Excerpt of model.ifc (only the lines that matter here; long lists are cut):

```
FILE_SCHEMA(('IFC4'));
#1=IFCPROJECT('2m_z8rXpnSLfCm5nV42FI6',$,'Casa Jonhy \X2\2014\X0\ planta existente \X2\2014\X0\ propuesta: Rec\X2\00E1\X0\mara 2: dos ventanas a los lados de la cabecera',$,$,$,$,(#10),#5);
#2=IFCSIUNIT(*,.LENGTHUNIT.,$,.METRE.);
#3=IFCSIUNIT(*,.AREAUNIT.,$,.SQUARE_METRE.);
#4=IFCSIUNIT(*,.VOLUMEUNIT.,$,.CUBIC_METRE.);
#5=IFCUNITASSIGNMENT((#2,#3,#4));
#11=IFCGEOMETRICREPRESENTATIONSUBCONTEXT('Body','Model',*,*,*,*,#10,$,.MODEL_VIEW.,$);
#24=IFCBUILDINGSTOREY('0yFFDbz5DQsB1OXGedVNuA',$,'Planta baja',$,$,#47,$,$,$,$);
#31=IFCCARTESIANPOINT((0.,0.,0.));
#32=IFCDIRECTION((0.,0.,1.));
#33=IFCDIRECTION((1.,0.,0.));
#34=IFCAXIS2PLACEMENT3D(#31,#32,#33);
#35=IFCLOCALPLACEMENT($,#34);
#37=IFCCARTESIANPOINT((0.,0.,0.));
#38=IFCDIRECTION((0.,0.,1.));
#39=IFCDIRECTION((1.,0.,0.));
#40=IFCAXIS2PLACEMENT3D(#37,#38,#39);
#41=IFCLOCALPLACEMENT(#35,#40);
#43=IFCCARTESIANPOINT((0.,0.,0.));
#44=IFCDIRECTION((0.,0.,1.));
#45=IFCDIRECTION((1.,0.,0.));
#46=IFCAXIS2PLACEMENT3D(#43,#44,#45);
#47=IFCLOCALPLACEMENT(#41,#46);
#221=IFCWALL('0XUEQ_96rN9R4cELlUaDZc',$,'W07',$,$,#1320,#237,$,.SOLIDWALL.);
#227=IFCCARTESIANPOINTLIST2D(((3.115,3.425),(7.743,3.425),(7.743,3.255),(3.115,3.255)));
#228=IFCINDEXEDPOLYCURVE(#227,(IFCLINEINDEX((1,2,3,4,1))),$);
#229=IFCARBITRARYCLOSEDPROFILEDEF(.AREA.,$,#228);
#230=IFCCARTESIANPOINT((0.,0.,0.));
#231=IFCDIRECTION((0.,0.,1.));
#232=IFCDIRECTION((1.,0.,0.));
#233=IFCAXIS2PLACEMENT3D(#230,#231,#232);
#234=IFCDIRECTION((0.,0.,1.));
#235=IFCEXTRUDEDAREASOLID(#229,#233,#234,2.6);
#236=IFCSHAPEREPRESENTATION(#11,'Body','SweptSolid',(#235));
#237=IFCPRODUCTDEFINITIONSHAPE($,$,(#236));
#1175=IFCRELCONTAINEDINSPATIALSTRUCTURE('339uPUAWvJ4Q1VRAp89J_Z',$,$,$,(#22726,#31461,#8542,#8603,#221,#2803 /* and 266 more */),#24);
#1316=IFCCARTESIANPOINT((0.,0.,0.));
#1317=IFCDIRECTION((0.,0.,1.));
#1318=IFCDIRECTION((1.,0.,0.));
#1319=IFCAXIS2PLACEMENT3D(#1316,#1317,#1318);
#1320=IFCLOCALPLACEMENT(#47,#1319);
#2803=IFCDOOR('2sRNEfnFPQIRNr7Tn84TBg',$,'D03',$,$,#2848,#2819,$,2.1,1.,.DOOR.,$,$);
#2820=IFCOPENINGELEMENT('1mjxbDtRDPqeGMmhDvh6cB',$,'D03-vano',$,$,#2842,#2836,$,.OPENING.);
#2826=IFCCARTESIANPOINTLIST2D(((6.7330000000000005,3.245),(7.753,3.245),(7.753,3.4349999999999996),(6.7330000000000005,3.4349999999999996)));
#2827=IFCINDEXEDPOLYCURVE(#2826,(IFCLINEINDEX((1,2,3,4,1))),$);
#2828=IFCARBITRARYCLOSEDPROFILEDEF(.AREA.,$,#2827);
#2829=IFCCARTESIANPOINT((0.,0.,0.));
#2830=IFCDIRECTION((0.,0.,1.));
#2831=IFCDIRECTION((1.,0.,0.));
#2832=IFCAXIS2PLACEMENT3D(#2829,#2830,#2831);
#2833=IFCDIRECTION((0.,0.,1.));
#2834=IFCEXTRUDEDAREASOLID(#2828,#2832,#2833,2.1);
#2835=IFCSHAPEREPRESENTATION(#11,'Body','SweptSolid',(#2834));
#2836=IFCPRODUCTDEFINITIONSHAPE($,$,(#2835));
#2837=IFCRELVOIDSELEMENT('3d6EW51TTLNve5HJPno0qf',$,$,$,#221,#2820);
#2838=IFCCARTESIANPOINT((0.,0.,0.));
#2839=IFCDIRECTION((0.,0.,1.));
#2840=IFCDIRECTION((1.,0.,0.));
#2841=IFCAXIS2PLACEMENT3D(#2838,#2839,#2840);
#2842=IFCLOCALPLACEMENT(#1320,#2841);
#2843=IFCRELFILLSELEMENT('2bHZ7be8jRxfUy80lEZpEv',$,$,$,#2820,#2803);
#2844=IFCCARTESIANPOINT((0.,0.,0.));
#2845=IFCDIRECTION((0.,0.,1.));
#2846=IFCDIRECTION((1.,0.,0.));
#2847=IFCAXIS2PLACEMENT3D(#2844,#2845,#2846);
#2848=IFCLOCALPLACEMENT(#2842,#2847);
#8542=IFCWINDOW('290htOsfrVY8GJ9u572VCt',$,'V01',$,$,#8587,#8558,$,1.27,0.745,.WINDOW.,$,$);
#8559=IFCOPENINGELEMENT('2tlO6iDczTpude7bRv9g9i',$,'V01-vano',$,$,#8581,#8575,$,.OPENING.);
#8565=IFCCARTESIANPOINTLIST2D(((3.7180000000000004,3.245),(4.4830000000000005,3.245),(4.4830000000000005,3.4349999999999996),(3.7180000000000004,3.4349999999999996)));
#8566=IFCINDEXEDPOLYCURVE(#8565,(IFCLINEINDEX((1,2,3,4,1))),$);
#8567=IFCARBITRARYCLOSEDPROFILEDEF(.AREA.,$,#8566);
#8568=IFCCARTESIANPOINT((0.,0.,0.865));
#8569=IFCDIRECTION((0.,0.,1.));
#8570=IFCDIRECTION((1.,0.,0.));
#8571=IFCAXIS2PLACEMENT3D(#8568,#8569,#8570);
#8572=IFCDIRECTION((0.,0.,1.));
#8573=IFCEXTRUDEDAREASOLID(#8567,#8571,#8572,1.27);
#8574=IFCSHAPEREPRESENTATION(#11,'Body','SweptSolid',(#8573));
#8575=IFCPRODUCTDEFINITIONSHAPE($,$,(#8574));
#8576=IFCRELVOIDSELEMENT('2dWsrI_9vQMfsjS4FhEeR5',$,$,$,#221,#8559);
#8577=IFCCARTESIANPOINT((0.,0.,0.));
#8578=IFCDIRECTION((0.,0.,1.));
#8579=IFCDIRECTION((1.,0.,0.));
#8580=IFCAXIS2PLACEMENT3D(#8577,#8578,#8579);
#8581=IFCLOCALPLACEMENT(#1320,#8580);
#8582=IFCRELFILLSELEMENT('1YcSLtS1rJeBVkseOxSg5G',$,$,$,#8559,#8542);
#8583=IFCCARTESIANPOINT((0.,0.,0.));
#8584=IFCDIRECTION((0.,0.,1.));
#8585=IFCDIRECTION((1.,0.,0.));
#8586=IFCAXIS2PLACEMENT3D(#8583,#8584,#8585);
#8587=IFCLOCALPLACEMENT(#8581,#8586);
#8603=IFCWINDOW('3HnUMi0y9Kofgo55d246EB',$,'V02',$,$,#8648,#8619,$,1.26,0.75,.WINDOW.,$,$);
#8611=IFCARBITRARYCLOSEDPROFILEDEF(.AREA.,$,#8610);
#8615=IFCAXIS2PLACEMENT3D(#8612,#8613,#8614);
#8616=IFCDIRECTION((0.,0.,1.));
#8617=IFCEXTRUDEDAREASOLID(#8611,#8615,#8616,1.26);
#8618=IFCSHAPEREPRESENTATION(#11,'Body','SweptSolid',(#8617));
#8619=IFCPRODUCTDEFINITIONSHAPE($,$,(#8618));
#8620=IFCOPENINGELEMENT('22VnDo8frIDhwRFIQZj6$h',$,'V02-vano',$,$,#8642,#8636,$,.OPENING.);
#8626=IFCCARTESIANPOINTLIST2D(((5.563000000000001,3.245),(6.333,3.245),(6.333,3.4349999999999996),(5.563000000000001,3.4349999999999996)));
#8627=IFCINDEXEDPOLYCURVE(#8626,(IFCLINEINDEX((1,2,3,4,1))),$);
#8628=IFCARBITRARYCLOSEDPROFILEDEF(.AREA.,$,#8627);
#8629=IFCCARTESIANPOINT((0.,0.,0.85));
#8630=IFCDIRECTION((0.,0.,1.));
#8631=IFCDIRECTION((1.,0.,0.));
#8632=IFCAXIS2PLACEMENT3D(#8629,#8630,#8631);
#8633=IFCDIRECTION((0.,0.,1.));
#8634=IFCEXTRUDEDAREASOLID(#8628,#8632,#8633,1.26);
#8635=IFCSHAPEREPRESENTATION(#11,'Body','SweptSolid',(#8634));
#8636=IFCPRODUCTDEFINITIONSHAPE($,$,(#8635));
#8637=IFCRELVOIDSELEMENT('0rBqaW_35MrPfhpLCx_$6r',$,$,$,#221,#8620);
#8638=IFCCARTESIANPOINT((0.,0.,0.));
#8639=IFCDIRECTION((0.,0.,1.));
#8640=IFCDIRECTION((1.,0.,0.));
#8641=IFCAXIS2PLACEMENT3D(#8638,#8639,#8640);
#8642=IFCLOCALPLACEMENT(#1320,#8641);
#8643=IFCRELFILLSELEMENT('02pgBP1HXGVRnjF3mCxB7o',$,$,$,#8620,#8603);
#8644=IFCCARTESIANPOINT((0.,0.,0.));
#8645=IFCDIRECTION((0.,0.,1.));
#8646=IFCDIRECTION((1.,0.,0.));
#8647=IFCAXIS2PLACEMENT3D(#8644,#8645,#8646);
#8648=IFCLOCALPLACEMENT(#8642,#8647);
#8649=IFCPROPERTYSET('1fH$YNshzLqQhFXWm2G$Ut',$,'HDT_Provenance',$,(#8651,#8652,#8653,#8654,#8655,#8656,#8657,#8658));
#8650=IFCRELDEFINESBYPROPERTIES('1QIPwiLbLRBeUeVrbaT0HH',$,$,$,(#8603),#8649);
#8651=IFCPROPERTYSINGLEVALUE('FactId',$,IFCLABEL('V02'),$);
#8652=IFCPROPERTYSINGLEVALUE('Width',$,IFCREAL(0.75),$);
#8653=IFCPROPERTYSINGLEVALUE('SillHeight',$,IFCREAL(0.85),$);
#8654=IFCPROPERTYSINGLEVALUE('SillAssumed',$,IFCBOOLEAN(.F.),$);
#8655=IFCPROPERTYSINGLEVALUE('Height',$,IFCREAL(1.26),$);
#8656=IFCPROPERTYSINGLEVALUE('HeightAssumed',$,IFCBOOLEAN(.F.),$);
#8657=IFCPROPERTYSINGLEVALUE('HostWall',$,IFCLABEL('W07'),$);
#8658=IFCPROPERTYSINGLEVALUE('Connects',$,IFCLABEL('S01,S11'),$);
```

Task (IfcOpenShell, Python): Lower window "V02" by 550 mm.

```python
import numpy as np
import ifcopenshell
import ifcopenshell.api.geometry
import ifcopenshell.api.pset
import ifcopenshell.util.element
import ifcopenshell.util.placement
import ifcopenshell.util.unit

model = ifcopenshell.open("model.ifc")
unit_scale = ifcopenshell.util.unit.calculate_unit_scale(model)

window = model.by_guid("3HnUMi0y9Kofgo55d246EB")
opening = window.FillsVoids[0].RelatingOpeningElement
dz = -0.55 / unit_scale

shift = np.array([0.0, 0.0, dz])
# The window is placed relative to its opening, so it follows when the opening moves.
matrix = ifcopenshell.util.placement.get_local_placement(opening.ObjectPlacement)
matrix[:3, 3] += shift
ifcopenshell.api.geometry.edit_object_placement(
    model, product=opening, matrix=matrix, is_si=False, should_transform_children=True
)

# Keep the stored heights in step.
pset = model.by_id(ifcopenshell.util.element.get_pset(window, "HDT_Provenance", should_inherit=False)["id"])
ifcopenshell.api.pset.edit_pset(model, pset=pset, properties={
    "SillHeight": model.create_entity("IfcReal", ifcopenshell.util.element.get_pset(window, "HDT_Provenance", "SillHeight") + dz),
})

print(f"moved by {dz * unit_scale:+.3f} m")

model.write("model_v2.ifc")
```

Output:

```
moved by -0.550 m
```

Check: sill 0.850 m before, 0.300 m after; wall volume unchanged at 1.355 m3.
